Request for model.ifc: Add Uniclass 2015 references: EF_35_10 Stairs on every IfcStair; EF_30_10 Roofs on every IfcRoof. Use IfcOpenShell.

First a look at what the model holds.

```python
import ifcopenshell

model = ifcopenshell.open("model.ifc")
print(model.schema)
print("classifications:", [c.Name for c in model.by_type("IfcClassification")])
for ifc_class in ("IfcDoor", "IfcRoof", "IfcStair", "IfcWall", "IfcWindow"):
    print(ifc_class, len(model.by_type(ifc_class)))
```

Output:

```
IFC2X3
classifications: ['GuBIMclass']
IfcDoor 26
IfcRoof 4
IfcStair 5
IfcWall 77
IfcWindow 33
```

```python
import ifcopenshell
import ifcopenshell.api.classification

model = ifcopenshell.open("model.ifc")

# IFC2X3 requires Source and Edition and has no link from the project to the system.
system = model.create_entity("IfcClassification", Source="NBS", Edition="2015", Name="Uniclass 2015")

codes = {
    "IfcStair": ("EF_35_10", "Stairs"),
    "IfcRoof": ("EF_30_10", "Roofs"),
}
for ifc_class, (code, name) in codes.items():
    products = model.by_type(ifc_class)
    ifcopenshell.api.classification.add_reference(
        model, products=products, classification=system, identification=code, name=name
    )
    print(code, len(products))

model.write("model_v2.ifc")
```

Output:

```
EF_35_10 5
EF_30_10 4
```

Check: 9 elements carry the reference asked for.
